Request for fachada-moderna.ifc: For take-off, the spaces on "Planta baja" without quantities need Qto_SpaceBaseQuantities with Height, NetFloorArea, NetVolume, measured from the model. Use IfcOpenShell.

First a look at what the model holds.

```python
import ifcopenshell
import ifcopenshell.util.element
import ifcopenshell.util.unit

model = ifcopenshell.open("fachada-moderna.ifc")
print(model.schema)
for unit_type in ("LENGTHUNIT", "AREAUNIT", "VOLUMEUNIT"):
    print(unit_type, ifcopenshell.util.unit.calculate_unit_scale(model, unit_type))
storey = next(s for s in model.by_type("IfcBuildingStorey") if s.Name == "Planta baja")
spaces = [e for e in ifcopenshell.util.element.get_decomposition(storey) if e.is_a("IfcSpace")]
for e in sorted(spaces, key=lambda e: e.id()):
    print(e.id(), e.is_a(), e.Name, list(ifcopenshell.util.element.get_psets(e, qtos_only=True)), sep=" | ")
```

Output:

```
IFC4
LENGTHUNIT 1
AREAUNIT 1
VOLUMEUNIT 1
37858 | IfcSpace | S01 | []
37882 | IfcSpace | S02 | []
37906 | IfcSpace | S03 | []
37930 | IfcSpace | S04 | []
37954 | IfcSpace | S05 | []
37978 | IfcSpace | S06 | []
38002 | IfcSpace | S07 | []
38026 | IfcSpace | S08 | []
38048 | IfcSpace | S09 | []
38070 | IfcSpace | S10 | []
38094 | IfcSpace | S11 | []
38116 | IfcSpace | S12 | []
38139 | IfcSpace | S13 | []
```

```python
import ifcopenshell
import ifcopenshell.api.pset
import ifcopenshell.geom
import ifcopenshell.util.element
import ifcopenshell.util.shape
import ifcopenshell.util.unit

model = ifcopenshell.open("fachada-moderna.ifc")
unit_scale = ifcopenshell.util.unit.calculate_unit_scale(model)
area_scale = ifcopenshell.util.unit.calculate_unit_scale(model, "AREAUNIT")
volume_scale = ifcopenshell.util.unit.calculate_unit_scale(model, "VOLUMEUNIT")
settings = ifcopenshell.geom.settings()

storey = next(s for s in model.by_type("IfcBuildingStorey") if s.Name == "Planta baja")
spaces = [e for e in ifcopenshell.util.element.get_decomposition(storey) if e.is_a("IfcSpace")]

for e in sorted(spaces, key=lambda e: e.id()):
    if ifcopenshell.util.element.get_psets(e, qtos_only=True, should_inherit=False):
        continue
    # Geometry comes back in metres, in the element's own axes.
    shape = ifcopenshell.geom.create_shape(settings, e)
    values = {
        "Height": ifcopenshell.util.shape.get_z(shape.geometry) / unit_scale,
        "NetFloorArea": ifcopenshell.util.shape.get_footprint_area(shape.geometry) / area_scale,
        "NetVolume": ifcopenshell.util.shape.get_volume(shape.geometry) / volume_scale,
    }
    qto = ifcopenshell.api.pset.add_qto(model, product=e, name="Qto_SpaceBaseQuantities")
    ifcopenshell.api.pset.edit_qto(model, qto=qto, properties=values)
    print(e.id(), {k: round(v, 3) for k, v in values.items()})

model.write("fachada-moderna_v2.ifc")
```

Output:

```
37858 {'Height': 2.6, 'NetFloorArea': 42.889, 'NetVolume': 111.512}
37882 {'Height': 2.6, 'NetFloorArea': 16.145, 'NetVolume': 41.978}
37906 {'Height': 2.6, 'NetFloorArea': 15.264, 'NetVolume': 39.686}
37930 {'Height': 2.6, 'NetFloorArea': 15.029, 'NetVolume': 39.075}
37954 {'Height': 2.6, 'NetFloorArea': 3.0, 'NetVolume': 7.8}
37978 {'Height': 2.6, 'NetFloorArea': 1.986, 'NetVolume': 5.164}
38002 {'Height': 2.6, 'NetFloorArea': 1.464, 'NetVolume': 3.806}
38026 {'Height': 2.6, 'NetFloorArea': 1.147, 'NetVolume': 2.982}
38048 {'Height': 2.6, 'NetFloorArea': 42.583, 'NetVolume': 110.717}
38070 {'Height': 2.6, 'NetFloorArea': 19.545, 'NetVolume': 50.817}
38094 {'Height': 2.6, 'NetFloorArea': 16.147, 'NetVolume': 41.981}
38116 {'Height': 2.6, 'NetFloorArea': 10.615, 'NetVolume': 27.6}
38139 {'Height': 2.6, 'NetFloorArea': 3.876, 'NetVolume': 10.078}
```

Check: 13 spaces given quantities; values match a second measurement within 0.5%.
